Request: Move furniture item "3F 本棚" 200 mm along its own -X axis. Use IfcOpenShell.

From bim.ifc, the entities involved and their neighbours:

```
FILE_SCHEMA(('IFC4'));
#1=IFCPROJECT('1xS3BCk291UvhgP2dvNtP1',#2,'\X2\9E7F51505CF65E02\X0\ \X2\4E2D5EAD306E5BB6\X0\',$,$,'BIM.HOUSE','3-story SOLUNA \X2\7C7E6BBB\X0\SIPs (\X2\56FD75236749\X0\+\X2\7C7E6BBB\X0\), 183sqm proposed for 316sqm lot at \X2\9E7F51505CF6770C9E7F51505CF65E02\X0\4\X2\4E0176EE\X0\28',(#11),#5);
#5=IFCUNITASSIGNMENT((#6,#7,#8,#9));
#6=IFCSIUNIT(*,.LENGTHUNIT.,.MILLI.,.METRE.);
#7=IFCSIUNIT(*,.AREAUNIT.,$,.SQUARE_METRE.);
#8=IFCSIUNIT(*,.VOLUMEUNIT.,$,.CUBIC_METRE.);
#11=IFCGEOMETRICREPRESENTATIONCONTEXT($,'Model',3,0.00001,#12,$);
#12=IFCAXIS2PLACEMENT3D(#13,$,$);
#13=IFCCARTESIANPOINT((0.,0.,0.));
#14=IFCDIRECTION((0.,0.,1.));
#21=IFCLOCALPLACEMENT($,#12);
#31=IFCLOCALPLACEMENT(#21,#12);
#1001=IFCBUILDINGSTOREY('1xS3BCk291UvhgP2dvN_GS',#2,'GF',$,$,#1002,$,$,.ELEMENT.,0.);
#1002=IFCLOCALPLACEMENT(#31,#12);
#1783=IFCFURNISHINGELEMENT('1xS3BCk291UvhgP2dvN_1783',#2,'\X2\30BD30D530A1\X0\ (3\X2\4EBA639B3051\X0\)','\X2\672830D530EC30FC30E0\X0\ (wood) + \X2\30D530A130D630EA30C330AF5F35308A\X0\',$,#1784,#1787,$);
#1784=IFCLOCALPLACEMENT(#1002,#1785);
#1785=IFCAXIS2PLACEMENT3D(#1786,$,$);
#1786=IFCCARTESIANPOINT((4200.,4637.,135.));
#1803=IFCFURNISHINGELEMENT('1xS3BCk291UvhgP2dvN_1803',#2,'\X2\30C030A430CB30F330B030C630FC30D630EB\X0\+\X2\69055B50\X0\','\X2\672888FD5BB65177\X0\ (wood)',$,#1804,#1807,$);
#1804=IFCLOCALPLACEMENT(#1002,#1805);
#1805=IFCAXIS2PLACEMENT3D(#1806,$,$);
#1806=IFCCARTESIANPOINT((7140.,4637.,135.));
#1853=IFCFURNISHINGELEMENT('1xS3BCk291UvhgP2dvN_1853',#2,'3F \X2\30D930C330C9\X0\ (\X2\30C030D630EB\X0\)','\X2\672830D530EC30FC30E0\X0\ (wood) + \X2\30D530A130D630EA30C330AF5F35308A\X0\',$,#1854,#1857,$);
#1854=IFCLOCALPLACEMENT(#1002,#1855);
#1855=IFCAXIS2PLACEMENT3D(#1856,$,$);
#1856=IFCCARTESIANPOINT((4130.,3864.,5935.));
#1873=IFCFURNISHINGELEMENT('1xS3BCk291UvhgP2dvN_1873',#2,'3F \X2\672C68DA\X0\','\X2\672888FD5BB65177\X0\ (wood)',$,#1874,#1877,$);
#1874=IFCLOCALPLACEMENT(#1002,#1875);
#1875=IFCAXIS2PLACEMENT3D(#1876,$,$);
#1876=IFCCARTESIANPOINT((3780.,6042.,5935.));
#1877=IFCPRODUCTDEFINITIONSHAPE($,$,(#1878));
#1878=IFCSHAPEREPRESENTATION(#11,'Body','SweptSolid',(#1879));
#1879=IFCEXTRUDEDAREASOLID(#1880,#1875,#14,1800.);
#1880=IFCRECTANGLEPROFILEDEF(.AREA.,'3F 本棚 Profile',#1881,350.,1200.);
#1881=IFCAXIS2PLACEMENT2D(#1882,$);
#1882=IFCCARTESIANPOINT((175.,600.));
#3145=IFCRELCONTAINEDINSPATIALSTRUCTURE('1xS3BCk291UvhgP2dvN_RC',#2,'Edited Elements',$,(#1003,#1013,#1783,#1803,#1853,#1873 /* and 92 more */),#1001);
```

```python
import ifcopenshell
import ifcopenshell.api.geometry
import ifcopenshell.util.placement
import ifcopenshell.util.unit

model = ifcopenshell.open("bim.ifc")
unit_scale = ifcopenshell.util.unit.calculate_unit_scale(model)

item = model.by_guid("1xS3BCk291UvhgP2dvN_1873")
matrix = ifcopenshell.util.placement.get_local_placement(item.ObjectPlacement)
matrix[:3, 3] -= matrix[:3, 0] * 0.2 / unit_scale
ifcopenshell.api.geometry.edit_object_placement(model, product=item, matrix=matrix, is_si=False)

print(ifcopenshell.util.placement.get_local_placement(item.ObjectPlacement).round(3) + 0.0)

model.write("bim-out.ifc")
```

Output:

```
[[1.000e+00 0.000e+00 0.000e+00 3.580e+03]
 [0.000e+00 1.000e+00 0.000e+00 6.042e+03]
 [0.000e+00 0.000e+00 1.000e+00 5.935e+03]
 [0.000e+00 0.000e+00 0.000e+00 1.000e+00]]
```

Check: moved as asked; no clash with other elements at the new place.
